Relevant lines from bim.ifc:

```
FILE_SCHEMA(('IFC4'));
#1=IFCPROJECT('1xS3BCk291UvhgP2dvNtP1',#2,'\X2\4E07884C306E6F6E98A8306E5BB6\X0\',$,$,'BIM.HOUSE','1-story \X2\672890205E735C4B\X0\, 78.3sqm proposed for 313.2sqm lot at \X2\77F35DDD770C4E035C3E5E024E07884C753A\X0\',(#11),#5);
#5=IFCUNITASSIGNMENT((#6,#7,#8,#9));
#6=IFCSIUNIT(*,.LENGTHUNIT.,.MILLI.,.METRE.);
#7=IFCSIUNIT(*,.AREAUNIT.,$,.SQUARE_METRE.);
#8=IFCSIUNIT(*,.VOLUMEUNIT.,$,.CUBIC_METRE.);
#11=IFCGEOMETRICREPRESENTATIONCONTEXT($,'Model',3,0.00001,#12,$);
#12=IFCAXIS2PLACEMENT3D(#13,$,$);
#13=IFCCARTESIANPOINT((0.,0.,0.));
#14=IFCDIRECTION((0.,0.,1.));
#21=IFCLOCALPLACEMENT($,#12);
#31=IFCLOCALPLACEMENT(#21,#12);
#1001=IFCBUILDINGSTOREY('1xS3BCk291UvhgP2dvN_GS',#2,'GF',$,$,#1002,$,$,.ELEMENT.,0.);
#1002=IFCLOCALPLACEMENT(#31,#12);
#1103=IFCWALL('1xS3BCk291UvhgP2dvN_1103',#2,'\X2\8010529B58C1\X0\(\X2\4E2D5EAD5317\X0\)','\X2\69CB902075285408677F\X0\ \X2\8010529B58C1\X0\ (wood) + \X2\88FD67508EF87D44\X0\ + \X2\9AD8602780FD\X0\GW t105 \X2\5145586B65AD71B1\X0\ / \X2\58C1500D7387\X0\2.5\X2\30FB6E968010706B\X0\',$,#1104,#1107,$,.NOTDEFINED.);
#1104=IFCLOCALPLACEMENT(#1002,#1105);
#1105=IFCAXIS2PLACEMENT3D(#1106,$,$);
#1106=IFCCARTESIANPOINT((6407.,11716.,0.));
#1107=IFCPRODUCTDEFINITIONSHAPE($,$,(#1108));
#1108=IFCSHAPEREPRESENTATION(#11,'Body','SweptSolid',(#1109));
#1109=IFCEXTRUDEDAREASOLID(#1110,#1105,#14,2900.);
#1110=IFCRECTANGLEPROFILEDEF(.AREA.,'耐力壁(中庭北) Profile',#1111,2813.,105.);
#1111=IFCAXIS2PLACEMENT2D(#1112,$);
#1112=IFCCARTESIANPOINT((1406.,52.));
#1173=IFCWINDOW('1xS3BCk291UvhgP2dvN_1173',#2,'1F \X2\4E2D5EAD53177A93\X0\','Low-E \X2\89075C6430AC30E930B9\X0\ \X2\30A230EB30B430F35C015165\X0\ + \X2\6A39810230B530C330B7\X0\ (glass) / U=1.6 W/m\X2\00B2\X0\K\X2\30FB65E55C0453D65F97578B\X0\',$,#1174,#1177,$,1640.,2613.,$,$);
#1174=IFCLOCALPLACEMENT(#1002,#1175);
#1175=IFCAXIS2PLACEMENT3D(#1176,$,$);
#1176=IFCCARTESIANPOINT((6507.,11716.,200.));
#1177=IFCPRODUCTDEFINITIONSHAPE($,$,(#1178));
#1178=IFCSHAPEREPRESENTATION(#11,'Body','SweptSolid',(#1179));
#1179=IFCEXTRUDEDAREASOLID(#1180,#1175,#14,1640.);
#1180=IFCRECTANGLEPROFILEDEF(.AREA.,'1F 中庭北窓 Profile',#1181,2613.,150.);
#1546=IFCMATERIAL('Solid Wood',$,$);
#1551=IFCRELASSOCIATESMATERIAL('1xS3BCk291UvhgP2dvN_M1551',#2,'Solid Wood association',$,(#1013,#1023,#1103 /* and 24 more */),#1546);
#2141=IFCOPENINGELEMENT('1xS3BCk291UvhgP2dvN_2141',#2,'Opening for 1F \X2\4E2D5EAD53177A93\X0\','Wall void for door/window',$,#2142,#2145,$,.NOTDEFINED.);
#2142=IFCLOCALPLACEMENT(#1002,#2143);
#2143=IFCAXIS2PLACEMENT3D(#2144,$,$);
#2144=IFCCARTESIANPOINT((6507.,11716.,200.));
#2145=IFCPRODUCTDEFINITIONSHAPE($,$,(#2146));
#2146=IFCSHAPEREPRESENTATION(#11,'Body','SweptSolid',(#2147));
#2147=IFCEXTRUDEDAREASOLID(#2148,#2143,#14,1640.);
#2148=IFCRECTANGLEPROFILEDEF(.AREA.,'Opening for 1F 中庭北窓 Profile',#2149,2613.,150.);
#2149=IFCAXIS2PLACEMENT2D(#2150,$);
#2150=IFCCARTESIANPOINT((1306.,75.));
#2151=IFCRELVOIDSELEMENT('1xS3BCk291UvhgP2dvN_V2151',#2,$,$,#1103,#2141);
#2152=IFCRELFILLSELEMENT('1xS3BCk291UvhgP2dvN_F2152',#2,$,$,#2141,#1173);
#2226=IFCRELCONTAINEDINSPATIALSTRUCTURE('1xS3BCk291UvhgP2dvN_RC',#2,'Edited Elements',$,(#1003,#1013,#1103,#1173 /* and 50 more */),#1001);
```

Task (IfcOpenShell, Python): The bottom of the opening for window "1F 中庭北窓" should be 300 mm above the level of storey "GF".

```python
import numpy as np
import ifcopenshell
import ifcopenshell.api.geometry
import ifcopenshell.geom
import ifcopenshell.util.element
import ifcopenshell.util.placement
import ifcopenshell.util.shape
import ifcopenshell.util.unit

model = ifcopenshell.open("bim.ifc")
unit_scale = ifcopenshell.util.unit.calculate_unit_scale(model)

window = model.by_guid("1xS3BCk291UvhgP2dvN_1173")
opening = window.FillsVoids[0].RelatingOpeningElement
storey = ifcopenshell.util.element.get_container(window, ifc_class="IfcBuildingStorey")
level = ifcopenshell.util.placement.get_local_placement(storey.ObjectPlacement)[2, 3]

# The opening's origin need not be at the sill, so measure its lowest point.
shape = ifcopenshell.geom.create_shape(ifcopenshell.geom.settings(), opening)
bottom = ifcopenshell.util.shape.get_shape_bottom_elevation(shape, shape.geometry) / unit_scale
dz = level + 0.3 / unit_scale - bottom

shift = np.array([0.0, 0.0, dz])
# The window is not placed relative to its opening, so move both.
for product in (opening, window):
    matrix = ifcopenshell.util.placement.get_local_placement(product.ObjectPlacement)
    matrix[:3, 3] += shift
    ifcopenshell.api.geometry.edit_object_placement(model, product=product, matrix=matrix, is_si=False)

print(f"moved by {dz * unit_scale:+.3f} m")

model.write("bim_rev.ifc")
```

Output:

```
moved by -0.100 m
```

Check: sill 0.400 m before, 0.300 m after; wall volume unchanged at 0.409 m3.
